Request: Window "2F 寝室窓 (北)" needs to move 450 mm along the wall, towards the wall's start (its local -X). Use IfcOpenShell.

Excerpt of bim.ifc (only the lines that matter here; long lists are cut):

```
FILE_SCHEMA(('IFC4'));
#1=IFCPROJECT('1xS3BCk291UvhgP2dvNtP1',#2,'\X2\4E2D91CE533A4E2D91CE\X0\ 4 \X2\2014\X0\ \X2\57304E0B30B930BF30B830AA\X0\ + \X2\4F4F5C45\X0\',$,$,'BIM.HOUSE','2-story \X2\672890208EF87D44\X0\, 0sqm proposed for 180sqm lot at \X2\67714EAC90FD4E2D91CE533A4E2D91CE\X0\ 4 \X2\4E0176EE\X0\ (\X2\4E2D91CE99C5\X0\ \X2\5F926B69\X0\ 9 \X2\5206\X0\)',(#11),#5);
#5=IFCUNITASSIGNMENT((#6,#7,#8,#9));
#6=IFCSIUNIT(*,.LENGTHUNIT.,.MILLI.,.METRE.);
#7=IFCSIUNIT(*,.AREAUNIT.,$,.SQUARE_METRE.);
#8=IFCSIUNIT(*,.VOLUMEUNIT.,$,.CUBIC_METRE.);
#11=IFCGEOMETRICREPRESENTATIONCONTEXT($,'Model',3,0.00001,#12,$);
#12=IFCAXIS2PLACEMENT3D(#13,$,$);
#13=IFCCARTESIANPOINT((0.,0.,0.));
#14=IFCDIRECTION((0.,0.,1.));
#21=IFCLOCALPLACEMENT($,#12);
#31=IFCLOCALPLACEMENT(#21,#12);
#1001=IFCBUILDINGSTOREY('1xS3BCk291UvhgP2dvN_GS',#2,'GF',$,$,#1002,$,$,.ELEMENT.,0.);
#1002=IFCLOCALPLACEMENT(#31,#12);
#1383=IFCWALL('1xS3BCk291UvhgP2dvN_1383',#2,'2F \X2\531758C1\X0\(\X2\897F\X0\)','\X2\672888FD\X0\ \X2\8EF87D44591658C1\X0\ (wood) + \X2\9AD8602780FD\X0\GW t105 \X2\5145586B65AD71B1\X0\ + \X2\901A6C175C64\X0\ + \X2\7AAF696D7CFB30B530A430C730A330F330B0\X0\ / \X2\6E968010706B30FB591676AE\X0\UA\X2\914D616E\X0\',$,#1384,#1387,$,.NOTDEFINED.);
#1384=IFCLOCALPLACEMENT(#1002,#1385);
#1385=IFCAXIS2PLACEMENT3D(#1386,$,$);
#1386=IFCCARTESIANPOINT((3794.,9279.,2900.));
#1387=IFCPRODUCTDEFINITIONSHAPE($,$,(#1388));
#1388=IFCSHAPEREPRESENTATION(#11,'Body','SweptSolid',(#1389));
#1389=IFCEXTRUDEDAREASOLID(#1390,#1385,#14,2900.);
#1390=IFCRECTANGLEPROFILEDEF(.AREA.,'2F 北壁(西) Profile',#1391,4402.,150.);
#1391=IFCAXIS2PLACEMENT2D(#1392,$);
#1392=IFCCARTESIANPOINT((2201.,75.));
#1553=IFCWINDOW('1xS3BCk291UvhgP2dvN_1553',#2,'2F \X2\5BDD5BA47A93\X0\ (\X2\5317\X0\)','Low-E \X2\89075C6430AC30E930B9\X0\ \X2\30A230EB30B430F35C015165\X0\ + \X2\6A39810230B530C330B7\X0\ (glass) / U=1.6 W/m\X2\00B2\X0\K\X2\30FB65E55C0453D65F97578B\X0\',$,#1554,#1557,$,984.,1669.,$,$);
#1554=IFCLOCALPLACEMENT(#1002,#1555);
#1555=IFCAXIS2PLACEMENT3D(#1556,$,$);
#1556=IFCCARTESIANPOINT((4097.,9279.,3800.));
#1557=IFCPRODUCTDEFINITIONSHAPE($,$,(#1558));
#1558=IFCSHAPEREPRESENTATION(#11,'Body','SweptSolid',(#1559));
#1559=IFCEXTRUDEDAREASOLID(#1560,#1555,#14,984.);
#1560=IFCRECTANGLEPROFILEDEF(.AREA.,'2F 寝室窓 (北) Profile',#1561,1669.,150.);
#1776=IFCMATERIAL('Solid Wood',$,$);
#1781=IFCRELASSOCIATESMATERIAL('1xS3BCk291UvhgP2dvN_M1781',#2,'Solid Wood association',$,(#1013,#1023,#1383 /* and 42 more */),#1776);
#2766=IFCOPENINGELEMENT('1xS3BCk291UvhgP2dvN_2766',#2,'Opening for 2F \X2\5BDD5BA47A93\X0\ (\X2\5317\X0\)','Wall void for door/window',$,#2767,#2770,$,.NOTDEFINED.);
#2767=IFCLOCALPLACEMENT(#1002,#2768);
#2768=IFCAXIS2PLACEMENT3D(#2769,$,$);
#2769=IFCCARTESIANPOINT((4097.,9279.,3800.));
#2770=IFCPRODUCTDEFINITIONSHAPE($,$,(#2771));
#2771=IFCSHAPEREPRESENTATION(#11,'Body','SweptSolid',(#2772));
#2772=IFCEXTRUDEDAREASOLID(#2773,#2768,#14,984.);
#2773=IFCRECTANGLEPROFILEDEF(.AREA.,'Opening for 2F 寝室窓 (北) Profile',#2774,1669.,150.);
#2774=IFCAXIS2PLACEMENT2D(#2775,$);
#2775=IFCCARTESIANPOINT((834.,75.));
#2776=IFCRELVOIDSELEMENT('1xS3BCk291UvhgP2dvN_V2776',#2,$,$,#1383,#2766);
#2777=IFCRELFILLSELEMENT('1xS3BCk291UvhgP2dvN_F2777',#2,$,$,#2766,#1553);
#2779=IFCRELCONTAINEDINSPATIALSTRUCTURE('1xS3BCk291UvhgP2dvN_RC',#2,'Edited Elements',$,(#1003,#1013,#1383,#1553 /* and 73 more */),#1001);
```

```python
import ifcopenshell
import ifcopenshell.api.geometry
import ifcopenshell.util.placement

model = ifcopenshell.open("bim.ifc")

window = model.by_guid("1xS3BCk291UvhgP2dvN_1553")
opening = window.FillsVoids[0].RelatingOpeningElement
wall = opening.VoidsElements[0].RelatingBuildingElement

wall_matrix = ifcopenshell.util.placement.get_local_placement(wall.ObjectPlacement)
shift = wall_matrix[:3, 0] * -450.0
before = ifcopenshell.util.placement.get_local_placement(window.ObjectPlacement)[:3, 3].copy()

# The window is not placed relative to its opening, so move both.
for product in (opening, window):
    matrix = ifcopenshell.util.placement.get_local_placement(product.ObjectPlacement)
    matrix[:3, 3] += shift
    ifcopenshell.api.geometry.edit_object_placement(model, product=product, matrix=matrix, is_si=False)

after = ifcopenshell.util.placement.get_local_placement(window.ObjectPlacement)[:3, 3]
print("window moved by", (after - before).round(3) + 0.0)

model.write("bim_rev.ifc")
```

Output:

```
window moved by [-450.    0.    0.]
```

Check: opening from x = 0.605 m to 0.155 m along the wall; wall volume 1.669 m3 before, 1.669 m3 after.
